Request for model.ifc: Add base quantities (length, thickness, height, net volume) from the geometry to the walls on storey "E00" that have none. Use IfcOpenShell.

First a look at what the model holds.

```python
import ifcopenshell
import ifcopenshell.util.element
import ifcopenshell.util.unit

model = ifcopenshell.open("model.ifc")
print(model.schema)
for unit_type in ("LENGTHUNIT", "AREAUNIT", "VOLUMEUNIT"):
    print(unit_type, ifcopenshell.util.unit.calculate_unit_scale(model, unit_type))
storey = next(s for s in model.by_type("IfcBuildingStorey") if s.Name == "E00")
walls = [e for e in ifcopenshell.util.element.get_decomposition(storey) if e.is_a("IfcWall")]
for e in sorted(walls, key=lambda e: e.id()):
    print(e.id(), e.is_a(), e.Name, list(ifcopenshell.util.element.get_psets(e, qtos_only=True)), sep=" | ")
```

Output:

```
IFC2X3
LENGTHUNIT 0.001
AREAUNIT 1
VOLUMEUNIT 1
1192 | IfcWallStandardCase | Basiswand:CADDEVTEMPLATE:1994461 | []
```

```python
import ifcopenshell
import ifcopenshell.api.pset
import ifcopenshell.geom
import ifcopenshell.util.element
import ifcopenshell.util.shape
import ifcopenshell.util.unit

model = ifcopenshell.open("model.ifc")
unit_scale = ifcopenshell.util.unit.calculate_unit_scale(model)
volume_scale = ifcopenshell.util.unit.calculate_unit_scale(model, "VOLUMEUNIT")
settings = ifcopenshell.geom.settings()

storey = next(s for s in model.by_type("IfcBuildingStorey") if s.Name == "E00")
walls = [e for e in ifcopenshell.util.element.get_decomposition(storey) if e.is_a("IfcWall")]

for e in sorted(walls, key=lambda e: e.id()):
    if ifcopenshell.util.element.get_psets(e, qtos_only=True, should_inherit=False):
        continue
    # Geometry comes back in metres, in the element's own axes.
    shape = ifcopenshell.geom.create_shape(settings, e)
    values = {
        "Length": ifcopenshell.util.shape.get_x(shape.geometry) / unit_scale,
        "Width": ifcopenshell.util.shape.get_y(shape.geometry) / unit_scale,
        "Height": ifcopenshell.util.shape.get_z(shape.geometry) / unit_scale,
        "NetVolume": ifcopenshell.util.shape.get_volume(shape.geometry) / volume_scale,
    }
    qto = ifcopenshell.api.pset.add_qto(model, product=e, name="BaseQuantities")
    ifcopenshell.api.pset.edit_qto(model, qto=qto, properties=values)
    print(e.id(), {k: round(v, 3) for k, v in values.items()})

model.write("model_updated.ifc")
```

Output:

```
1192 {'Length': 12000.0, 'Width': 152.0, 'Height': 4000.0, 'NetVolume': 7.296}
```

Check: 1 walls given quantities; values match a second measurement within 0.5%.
